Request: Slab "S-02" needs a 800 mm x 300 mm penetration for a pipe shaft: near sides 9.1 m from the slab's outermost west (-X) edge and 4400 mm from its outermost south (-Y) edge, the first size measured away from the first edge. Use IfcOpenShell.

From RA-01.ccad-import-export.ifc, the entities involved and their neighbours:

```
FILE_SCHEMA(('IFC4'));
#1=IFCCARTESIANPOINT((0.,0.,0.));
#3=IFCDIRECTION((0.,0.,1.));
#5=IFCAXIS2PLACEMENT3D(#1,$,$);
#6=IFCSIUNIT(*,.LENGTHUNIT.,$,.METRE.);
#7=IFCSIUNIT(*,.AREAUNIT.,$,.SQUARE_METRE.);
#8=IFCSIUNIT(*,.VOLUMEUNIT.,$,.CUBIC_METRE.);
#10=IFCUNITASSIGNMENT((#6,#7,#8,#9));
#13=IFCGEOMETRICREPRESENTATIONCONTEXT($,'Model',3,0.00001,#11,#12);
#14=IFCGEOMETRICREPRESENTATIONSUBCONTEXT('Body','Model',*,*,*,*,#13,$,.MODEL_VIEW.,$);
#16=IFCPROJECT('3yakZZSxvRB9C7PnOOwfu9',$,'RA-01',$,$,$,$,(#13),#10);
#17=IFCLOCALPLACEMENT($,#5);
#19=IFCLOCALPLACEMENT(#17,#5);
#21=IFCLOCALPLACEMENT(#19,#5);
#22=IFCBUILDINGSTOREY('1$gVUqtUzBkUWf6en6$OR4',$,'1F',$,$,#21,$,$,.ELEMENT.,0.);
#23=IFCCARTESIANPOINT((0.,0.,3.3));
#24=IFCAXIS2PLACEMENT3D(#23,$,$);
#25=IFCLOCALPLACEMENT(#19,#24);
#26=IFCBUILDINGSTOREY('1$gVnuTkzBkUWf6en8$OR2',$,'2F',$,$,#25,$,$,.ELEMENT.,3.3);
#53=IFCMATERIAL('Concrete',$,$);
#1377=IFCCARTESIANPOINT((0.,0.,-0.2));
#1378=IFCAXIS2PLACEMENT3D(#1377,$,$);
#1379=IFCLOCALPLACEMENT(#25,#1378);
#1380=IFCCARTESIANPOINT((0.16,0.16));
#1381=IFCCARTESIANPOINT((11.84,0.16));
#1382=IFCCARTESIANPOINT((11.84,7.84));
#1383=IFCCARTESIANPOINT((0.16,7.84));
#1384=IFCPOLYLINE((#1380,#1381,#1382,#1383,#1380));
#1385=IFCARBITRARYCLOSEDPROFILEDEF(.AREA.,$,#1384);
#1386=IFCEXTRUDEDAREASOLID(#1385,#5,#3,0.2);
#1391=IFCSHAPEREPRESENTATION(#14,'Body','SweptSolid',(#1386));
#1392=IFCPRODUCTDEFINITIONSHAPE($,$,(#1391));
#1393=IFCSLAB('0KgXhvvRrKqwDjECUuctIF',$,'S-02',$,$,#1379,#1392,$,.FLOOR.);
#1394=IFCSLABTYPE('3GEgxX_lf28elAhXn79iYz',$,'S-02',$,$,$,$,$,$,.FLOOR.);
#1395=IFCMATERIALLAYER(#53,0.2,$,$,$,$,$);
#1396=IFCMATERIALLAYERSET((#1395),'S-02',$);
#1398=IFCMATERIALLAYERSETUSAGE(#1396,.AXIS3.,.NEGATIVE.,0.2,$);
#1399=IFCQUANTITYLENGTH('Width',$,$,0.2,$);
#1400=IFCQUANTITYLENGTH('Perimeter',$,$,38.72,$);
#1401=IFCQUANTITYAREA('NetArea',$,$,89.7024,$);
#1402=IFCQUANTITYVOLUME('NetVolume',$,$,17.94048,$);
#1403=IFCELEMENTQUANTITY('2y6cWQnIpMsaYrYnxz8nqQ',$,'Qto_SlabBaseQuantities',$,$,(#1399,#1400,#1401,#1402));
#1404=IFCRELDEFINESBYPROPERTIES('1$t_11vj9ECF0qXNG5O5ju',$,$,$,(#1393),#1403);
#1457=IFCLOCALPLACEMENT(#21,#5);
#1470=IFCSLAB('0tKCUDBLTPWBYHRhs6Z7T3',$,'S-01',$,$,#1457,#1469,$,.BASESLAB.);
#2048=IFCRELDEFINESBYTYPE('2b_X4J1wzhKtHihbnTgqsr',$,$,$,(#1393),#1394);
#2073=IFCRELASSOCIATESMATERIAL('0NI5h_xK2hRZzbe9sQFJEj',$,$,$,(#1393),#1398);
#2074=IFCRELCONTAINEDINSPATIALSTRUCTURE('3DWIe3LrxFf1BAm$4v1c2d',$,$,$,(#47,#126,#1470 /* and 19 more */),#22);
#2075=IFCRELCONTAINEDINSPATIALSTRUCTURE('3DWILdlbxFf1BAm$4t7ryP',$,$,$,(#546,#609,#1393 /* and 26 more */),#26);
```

```python
import numpy as np
import ifcopenshell
import ifcopenshell.api.feature
import ifcopenshell.api.geometry
import ifcopenshell.api.pset
import ifcopenshell.api.root
import ifcopenshell.geom
import ifcopenshell.util.element
import ifcopenshell.util.placement
import ifcopenshell.util.representation
import ifcopenshell.util.shape
import ifcopenshell.util.unit

model = ifcopenshell.open("RA-01.ccad-import-export.ifc")
unit_scale = ifcopenshell.util.unit.calculate_unit_scale(model)
area_scale = ifcopenshell.util.unit.calculate_unit_scale(model, "AREAUNIT")
volume_scale = ifcopenshell.util.unit.calculate_unit_scale(model, "VOLUMEUNIT")
settings = ifcopenshell.geom.settings()


def volume(element):
    """Net volume in cubic metres, openings subtracted."""
    shape = ifcopenshell.geom.create_shape(settings, element)
    return ifcopenshell.util.shape.get_volume(shape.geometry)


slab = model.by_guid("0KgXhvvRrKqwDjECUuctIF")
before = volume(slab)

# Extent in the slab's own axes, in metres. The edges named are its -X and -Y sides.
slab_shape = ifcopenshell.geom.create_shape(settings, slab)
vertices = ifcopenshell.util.shape.get_vertices(slab_shape.geometry)
x_min, y_min, bottom = vertices.min(axis=0)
top = vertices[:, 2].max()

opening = ifcopenshell.api.root.create_entity(model, ifc_class="IfcOpeningElement", name="Pipe shaft opening", predefined_type="OPENING")
context = ifcopenshell.util.representation.get_context(model, "Model", "Body", "MODEL_VIEW")
width, depth = 0.8, 0.3
outline = [(0.0, 0.0), (width, 0.0), (width, depth), (0.0, depth), (0.0, 0.0)]
# Overshoot both faces by 50 mm so the cut is clean.
shape = ifcopenshell.api.geometry.add_slab_representation(
    model, context=context, depth=top - bottom + 0.1, polyline=outline
)
ifcopenshell.api.geometry.assign_representation(model, product=opening, representation=shape)

matrix = ifcopenshell.util.placement.get_local_placement(slab.ObjectPlacement)
matrix[:, 3] = matrix @ np.append(np.array([x_min + 9.1, y_min + 4.4, bottom - 0.05]) / unit_scale, 1.0)
ifcopenshell.api.geometry.edit_object_placement(model, product=opening, matrix=matrix, is_si=False)
ifcopenshell.api.feature.add_feature(model, feature=opening, element=slab)

after = volume(slab)

# Update the slab's stored quantities.
qto = model.by_id(ifcopenshell.util.element.get_pset(slab, "Qto_SlabBaseQuantities", should_inherit=False)["id"])
ifcopenshell.api.pset.edit_qto(model, qto=qto, properties={
    "NetArea": after / (top - bottom) / area_scale,
    "NetVolume": after / volume_scale,
})

print(f"slab volume {before:.3f} -> {after:.3f} m3")

model.write("RA-01.ccad-import-export_rev.ifc")
```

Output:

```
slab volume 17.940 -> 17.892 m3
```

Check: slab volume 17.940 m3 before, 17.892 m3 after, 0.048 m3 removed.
